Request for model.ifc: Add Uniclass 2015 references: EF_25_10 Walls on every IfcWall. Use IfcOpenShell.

First a look at what the model holds.

```python
import ifcopenshell

model = ifcopenshell.open("model.ifc")
print(model.schema)
print("classifications:", [c.Name for c in model.by_type("IfcClassification")])
for ifc_class in ("IfcDoor", "IfcRoof", "IfcStair", "IfcWall", "IfcWindow"):
    print(ifc_class, len(model.by_type(ifc_class)))
```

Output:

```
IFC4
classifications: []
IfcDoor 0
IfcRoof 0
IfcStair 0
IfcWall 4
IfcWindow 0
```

```python
import ifcopenshell
import ifcopenshell.api.classification

model = ifcopenshell.open("model.ifc")

system = ifcopenshell.api.classification.add_classification(model, classification="Uniclass 2015")

codes = {
    "IfcWall": ("EF_25_10", "Walls"),
}
for ifc_class, (code, name) in codes.items():
    products = model.by_type(ifc_class)
    ifcopenshell.api.classification.add_reference(
        model, products=products, classification=system, identification=code, name=name
    )
    print(code, len(products))

model.write("model_rev.ifc")
```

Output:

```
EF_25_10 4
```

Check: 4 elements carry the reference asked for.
